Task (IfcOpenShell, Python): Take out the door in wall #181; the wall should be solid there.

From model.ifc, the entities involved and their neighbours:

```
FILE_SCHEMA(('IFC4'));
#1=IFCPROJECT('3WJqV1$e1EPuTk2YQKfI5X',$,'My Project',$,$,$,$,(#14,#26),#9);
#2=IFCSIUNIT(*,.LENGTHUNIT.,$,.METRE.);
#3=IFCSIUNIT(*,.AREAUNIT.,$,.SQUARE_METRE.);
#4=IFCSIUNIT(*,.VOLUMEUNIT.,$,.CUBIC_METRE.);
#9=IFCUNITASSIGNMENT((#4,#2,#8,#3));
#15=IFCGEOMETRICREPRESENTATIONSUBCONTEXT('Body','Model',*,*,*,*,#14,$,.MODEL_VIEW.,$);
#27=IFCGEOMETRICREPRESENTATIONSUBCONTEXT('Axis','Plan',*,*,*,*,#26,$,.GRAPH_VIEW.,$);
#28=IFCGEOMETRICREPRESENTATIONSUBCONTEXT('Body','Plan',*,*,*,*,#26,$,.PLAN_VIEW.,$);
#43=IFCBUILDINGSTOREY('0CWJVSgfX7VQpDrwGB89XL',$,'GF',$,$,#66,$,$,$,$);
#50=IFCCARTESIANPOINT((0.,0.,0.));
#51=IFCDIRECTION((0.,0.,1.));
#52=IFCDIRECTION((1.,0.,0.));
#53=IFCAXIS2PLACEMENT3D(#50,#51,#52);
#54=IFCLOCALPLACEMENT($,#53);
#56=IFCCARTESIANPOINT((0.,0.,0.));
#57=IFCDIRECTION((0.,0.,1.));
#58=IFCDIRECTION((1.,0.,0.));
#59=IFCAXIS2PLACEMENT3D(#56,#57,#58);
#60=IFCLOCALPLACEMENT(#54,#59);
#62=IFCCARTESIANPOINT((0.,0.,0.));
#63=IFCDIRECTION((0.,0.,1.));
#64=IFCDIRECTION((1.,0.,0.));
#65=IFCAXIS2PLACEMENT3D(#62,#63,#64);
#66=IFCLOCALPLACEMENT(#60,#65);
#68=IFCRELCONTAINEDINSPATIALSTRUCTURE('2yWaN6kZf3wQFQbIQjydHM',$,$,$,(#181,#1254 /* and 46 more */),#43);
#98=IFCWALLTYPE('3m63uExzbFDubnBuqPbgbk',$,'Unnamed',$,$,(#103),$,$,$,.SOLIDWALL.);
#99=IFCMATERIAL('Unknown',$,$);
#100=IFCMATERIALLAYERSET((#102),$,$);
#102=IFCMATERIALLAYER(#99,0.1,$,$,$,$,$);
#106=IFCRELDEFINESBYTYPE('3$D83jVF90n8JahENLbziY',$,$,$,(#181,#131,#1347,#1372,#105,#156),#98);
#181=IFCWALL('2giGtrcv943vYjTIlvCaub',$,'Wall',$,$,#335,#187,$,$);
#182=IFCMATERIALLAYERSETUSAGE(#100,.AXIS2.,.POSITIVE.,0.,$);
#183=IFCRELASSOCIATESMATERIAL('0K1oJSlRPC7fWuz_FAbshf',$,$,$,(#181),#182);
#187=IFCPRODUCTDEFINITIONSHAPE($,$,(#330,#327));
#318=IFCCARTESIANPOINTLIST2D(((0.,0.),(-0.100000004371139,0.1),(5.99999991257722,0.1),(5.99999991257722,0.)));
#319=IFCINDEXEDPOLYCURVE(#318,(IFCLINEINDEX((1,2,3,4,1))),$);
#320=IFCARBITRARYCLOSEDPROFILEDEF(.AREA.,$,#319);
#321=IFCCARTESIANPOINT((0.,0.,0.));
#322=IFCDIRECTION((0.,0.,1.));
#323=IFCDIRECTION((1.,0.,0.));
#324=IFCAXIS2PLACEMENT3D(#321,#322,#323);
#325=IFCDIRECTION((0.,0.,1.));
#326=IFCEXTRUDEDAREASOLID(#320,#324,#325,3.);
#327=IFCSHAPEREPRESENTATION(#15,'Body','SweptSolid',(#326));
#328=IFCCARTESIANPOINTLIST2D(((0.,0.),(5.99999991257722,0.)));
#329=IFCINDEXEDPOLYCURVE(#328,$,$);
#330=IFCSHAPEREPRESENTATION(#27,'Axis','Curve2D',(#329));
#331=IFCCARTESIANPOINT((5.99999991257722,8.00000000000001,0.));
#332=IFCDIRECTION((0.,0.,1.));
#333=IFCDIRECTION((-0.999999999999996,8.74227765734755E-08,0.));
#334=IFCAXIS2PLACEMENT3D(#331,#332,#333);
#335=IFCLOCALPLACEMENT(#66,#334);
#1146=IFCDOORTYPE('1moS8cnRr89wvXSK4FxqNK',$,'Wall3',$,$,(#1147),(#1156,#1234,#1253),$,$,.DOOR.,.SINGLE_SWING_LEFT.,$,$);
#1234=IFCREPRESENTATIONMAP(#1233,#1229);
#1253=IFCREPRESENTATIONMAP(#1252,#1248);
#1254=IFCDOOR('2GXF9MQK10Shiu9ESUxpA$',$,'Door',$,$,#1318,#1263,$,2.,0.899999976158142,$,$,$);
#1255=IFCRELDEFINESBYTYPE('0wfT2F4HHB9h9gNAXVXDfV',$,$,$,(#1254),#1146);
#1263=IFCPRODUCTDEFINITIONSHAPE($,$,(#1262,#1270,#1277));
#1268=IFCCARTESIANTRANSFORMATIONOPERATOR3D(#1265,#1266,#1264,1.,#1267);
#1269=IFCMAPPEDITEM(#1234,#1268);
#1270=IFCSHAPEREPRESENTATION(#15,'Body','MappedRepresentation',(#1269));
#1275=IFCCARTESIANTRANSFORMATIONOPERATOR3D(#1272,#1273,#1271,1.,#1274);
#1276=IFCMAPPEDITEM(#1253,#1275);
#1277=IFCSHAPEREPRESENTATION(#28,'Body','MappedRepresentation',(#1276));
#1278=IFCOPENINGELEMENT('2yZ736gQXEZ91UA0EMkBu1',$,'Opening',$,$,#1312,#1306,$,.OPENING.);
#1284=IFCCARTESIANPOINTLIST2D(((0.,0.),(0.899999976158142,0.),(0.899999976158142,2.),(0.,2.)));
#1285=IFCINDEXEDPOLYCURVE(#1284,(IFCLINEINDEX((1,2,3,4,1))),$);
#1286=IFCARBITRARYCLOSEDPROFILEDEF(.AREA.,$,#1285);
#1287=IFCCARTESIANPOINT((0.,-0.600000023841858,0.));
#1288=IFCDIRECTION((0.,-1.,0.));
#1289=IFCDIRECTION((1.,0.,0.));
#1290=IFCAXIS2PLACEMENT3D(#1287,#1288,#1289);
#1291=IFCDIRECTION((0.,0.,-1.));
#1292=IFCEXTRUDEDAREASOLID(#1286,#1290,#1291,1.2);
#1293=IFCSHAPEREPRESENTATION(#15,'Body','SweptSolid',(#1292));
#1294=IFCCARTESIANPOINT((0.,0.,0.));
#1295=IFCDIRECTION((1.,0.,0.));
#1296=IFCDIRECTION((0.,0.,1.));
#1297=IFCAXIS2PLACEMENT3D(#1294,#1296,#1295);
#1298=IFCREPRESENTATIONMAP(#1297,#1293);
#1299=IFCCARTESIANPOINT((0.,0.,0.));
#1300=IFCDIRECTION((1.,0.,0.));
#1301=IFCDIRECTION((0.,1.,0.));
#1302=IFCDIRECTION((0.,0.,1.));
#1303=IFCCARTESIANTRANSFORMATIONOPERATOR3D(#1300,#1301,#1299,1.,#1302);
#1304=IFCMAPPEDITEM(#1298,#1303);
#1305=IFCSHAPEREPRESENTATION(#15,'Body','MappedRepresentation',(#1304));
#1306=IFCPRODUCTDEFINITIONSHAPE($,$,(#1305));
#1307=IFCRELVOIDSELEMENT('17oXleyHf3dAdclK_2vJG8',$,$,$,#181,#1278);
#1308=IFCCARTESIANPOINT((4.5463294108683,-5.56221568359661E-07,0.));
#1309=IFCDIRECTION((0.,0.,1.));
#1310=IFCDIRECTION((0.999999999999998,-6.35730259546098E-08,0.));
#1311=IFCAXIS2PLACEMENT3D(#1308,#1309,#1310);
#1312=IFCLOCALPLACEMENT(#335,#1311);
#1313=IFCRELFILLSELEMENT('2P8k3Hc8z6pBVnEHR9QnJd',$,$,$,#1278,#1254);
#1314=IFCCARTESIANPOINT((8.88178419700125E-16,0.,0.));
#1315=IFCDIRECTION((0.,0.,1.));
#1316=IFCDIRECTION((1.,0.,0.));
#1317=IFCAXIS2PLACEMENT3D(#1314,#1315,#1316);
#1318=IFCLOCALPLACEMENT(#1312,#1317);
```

```python
import ifcopenshell
import ifcopenshell.api.feature
import ifcopenshell.api.root
import ifcopenshell.geom
import ifcopenshell.util.shape

model = ifcopenshell.open("model.ifc")
settings = ifcopenshell.geom.settings()


def volume(element):
    """Net volume in cubic metres, openings subtracted."""
    shape = ifcopenshell.geom.create_shape(settings, element)
    return ifcopenshell.util.shape.get_volume(shape.geometry)


door = model.by_guid("2GXF9MQK10Shiu9ESUxpA$")
opening = door.FillsVoids[0].RelatingOpeningElement
wall = opening.VoidsElements[0].RelatingBuildingElement
before = volume(wall)

ifcopenshell.api.root.remove_product(model, product=door)
ifcopenshell.api.feature.remove_feature(model, feature=opening)

after = volume(wall)

print(f"wall volume {before:.3f} -> {after:.3f} m3")

model.write("model_updated.ifc")
```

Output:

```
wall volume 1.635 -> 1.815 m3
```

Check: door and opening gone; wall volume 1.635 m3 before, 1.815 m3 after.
